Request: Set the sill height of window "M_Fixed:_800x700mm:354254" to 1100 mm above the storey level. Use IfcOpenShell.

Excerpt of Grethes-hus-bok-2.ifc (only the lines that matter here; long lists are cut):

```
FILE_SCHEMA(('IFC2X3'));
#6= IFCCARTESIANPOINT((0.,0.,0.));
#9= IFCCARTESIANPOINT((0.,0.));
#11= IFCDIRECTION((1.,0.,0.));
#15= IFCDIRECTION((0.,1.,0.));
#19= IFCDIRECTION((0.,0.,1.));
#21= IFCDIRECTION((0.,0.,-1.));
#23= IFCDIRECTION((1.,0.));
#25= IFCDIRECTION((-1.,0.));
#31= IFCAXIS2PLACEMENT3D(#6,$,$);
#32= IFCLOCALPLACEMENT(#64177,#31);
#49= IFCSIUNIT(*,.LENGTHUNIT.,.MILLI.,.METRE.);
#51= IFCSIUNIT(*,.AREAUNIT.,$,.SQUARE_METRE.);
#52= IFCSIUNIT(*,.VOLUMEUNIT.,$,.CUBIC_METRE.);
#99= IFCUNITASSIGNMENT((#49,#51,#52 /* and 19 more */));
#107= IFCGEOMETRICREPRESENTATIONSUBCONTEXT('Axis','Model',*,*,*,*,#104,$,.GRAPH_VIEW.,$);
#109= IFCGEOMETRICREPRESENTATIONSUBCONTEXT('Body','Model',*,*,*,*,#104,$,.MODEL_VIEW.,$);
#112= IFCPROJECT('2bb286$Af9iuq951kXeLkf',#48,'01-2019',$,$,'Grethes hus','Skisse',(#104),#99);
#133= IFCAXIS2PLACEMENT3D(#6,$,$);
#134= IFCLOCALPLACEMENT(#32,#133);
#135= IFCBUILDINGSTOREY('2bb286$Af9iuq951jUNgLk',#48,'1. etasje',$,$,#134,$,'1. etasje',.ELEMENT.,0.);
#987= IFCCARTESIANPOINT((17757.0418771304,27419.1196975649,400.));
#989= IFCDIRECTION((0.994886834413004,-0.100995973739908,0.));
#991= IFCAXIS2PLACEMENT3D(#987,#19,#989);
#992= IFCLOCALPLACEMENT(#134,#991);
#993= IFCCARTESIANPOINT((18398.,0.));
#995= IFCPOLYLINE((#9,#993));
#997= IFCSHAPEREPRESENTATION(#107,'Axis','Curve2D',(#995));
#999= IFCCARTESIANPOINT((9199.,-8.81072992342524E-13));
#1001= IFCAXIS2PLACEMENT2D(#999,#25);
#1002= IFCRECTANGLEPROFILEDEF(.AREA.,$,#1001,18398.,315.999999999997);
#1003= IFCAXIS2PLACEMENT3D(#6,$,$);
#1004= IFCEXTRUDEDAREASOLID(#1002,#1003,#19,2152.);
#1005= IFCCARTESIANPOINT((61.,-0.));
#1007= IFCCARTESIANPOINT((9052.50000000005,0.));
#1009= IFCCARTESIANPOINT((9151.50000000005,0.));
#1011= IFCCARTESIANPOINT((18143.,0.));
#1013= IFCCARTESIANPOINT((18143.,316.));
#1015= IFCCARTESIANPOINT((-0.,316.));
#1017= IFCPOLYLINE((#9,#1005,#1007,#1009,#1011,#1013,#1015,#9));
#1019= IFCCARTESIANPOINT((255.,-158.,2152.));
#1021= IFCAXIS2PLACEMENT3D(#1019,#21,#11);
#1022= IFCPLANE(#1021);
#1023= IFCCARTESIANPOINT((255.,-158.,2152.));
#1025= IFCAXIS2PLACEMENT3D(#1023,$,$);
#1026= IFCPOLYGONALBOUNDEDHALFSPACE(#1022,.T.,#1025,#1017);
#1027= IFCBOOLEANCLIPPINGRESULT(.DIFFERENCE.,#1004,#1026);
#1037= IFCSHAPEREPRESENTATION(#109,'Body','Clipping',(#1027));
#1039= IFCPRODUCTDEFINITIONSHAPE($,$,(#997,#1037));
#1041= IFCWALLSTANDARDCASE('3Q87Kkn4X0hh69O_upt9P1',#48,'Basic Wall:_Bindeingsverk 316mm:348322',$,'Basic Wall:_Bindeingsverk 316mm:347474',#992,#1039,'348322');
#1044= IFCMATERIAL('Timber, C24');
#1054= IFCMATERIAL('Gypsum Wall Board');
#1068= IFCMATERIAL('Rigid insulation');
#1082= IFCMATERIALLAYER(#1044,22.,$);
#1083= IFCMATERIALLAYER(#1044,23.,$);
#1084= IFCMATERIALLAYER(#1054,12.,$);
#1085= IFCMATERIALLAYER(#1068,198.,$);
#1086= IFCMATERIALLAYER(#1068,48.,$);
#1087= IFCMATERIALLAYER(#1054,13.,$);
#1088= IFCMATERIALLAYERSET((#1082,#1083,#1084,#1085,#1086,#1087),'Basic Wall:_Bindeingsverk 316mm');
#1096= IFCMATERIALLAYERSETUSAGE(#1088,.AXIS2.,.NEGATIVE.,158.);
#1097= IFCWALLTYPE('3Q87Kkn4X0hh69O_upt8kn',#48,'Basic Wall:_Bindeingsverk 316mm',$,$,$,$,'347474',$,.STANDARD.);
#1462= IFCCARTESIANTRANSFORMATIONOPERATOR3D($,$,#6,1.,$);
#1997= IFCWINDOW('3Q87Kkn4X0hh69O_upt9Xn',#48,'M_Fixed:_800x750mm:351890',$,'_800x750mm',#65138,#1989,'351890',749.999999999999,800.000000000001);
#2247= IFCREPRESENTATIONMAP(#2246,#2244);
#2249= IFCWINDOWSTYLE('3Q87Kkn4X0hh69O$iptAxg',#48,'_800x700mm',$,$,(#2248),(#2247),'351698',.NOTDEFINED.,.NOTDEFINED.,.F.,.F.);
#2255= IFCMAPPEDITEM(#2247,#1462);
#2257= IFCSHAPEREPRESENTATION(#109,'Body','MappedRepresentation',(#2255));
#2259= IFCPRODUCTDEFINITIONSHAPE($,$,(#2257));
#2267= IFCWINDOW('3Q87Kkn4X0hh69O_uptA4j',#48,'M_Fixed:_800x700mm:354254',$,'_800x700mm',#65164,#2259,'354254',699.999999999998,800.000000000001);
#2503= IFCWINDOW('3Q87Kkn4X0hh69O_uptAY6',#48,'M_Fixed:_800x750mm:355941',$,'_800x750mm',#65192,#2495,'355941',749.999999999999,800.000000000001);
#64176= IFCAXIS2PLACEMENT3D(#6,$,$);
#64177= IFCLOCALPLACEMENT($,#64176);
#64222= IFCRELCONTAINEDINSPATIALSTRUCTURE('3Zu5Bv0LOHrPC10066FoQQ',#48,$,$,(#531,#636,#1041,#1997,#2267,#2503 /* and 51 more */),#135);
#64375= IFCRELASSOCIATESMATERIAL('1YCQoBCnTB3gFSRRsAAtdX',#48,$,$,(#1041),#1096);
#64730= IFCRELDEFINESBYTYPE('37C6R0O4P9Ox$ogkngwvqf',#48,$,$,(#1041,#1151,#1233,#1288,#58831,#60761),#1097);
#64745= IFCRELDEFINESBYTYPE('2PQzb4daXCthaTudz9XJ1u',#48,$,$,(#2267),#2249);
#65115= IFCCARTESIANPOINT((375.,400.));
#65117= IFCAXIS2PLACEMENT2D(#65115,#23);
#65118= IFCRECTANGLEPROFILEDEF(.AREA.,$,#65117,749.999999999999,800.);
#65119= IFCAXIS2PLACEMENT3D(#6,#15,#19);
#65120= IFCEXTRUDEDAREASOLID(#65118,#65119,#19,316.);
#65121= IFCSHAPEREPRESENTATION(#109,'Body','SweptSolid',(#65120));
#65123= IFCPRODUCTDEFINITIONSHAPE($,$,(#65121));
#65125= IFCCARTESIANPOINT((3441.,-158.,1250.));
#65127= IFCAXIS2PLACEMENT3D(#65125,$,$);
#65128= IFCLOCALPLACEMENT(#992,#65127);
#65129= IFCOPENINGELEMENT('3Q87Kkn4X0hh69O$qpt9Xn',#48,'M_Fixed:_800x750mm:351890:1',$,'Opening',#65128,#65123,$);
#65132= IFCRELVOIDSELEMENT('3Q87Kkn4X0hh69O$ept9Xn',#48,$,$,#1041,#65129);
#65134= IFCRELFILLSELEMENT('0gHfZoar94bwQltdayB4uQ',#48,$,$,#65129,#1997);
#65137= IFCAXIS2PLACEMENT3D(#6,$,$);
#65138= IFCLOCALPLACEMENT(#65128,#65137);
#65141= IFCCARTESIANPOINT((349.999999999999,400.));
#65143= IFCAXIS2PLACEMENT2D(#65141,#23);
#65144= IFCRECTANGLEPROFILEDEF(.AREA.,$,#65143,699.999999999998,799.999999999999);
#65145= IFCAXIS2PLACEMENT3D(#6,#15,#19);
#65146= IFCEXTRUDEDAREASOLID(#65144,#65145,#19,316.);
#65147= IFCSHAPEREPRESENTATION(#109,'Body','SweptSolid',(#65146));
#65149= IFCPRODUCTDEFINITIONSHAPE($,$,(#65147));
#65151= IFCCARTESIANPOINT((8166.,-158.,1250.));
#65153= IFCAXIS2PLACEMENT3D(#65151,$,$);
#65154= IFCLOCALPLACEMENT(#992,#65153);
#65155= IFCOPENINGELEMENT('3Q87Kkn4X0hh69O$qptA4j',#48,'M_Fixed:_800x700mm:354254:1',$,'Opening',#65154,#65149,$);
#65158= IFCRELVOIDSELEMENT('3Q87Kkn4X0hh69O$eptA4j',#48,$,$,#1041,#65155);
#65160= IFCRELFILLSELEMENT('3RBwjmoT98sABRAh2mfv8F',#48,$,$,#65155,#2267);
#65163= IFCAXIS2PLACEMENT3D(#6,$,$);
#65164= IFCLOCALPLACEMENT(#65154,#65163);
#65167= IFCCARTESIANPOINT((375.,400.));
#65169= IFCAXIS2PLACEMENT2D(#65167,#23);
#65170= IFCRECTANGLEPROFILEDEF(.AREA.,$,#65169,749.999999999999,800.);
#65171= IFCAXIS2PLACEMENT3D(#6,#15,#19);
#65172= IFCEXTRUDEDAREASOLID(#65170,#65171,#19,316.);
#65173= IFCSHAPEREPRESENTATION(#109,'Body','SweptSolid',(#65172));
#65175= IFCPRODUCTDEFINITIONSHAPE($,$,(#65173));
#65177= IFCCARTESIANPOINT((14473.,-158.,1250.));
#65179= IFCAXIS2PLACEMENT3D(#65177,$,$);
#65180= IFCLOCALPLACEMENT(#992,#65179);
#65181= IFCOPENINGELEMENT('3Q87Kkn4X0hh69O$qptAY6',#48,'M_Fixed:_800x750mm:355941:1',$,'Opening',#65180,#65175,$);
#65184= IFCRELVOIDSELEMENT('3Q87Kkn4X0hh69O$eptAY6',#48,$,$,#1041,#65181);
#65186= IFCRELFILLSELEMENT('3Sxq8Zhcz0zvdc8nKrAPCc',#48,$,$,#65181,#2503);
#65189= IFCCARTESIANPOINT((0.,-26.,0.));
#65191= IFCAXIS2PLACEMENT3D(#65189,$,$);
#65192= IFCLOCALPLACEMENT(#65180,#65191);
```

```python
import numpy as np
import ifcopenshell
import ifcopenshell.api.geometry
import ifcopenshell.geom
import ifcopenshell.util.element
import ifcopenshell.util.placement
import ifcopenshell.util.shape
import ifcopenshell.util.unit

model = ifcopenshell.open("Grethes-hus-bok-2.ifc")
unit_scale = ifcopenshell.util.unit.calculate_unit_scale(model)

window = model.by_guid("3Q87Kkn4X0hh69O_uptA4j")
opening = window.FillsVoids[0].RelatingOpeningElement
storey = ifcopenshell.util.element.get_container(window, ifc_class="IfcBuildingStorey")
level = ifcopenshell.util.placement.get_local_placement(storey.ObjectPlacement)[2, 3]

# The opening's origin need not be at the sill, so measure its lowest point.
shape = ifcopenshell.geom.create_shape(ifcopenshell.geom.settings(), opening)
bottom = ifcopenshell.util.shape.get_shape_bottom_elevation(shape, shape.geometry) / unit_scale
dz = level + 1.1 / unit_scale - bottom

shift = np.array([0.0, 0.0, dz])
# The window is placed relative to its opening, so it follows when the opening moves.
matrix = ifcopenshell.util.placement.get_local_placement(opening.ObjectPlacement)
matrix[:3, 3] += shift
ifcopenshell.api.geometry.edit_object_placement(
    model, product=opening, matrix=matrix, is_si=False, should_transform_children=True
)

print(f"moved by {dz * unit_scale:+.3f} m")

model.write("Grethes-hus-bok-2_v2.ifc")
```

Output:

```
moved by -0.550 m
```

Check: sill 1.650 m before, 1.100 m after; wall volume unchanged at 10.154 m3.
